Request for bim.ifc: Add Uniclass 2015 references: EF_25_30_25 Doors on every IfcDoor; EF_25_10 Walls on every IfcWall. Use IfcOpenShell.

First a look at what the model holds.

```python
import ifcopenshell

model = ifcopenshell.open("bim.ifc")
print(model.schema)
print("classifications:", [c.Name for c in model.by_type("IfcClassification")])
for ifc_class in ("IfcDoor", "IfcRoof", "IfcStair", "IfcWall", "IfcWindow"):
    print(ifc_class, len(model.by_type(ifc_class)))
```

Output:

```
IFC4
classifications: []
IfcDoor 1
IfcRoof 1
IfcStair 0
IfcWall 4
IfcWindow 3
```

```python
import ifcopenshell
import ifcopenshell.api.classification

model = ifcopenshell.open("bim.ifc")

system = ifcopenshell.api.classification.add_classification(model, classification="Uniclass 2015")

codes = {
    "IfcDoor": ("EF_25_30_25", "Doors"),
    "IfcWall": ("EF_25_10", "Walls"),
}
for ifc_class, (code, name) in codes.items():
    products = model.by_type(ifc_class)
    ifcopenshell.api.classification.add_reference(
        model, products=products, classification=system, identification=code, name=name
    )
    print(code, len(products))

model.write("bim_edited.ifc")
```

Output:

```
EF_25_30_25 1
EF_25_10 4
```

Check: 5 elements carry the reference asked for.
